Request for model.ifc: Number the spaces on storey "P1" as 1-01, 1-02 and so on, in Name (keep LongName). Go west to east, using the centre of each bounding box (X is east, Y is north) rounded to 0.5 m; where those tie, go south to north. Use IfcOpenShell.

First a look at what the model holds.

```python
import ifcopenshell
import ifcopenshell.util.element
import ifcopenshell.util.placement

model = ifcopenshell.open("model.ifc")
print(model.schema)
storey = next(s for s in model.by_type("IfcBuildingStorey") if s.Name == "P1")
spaces = [e for e in ifcopenshell.util.element.get_decomposition(storey) if e.is_a("IfcSpace")]
for e in sorted(spaces, key=lambda e: e.id()):
    origin = ifcopenshell.util.placement.get_local_placement(e.ObjectPlacement)[:3, 3]
    print(e.id(), e.Name, e.LongName, origin.round(2) + 0.0, sep=" | ")
```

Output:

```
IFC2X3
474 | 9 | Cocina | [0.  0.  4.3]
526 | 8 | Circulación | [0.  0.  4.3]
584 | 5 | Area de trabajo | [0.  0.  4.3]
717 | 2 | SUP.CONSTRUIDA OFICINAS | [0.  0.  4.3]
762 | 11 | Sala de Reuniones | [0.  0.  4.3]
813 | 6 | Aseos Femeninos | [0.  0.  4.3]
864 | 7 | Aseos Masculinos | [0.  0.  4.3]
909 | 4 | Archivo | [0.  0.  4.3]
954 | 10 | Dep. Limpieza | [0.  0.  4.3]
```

```python
import ifcopenshell
import ifcopenshell.geom
import ifcopenshell.util.element
import ifcopenshell.util.shape

model = ifcopenshell.open("model.ifc")
settings = ifcopenshell.geom.settings()
settings.set("use-world-coords", True)


def centre(element):
    shape = ifcopenshell.geom.create_shape(settings, element)
    return ifcopenshell.util.shape.get_bbox_centroid(shape.geometry)


storey = next(s for s in model.by_type("IfcBuildingStorey") if s.Name == "P1")
spaces = [e for e in ifcopenshell.util.element.get_decomposition(storey) if e.is_a("IfcSpace")]

# Insertion points can sit at a corner or the storey origin, so sort by the geometry (in metres).
centres = {e: centre(e) for e in spaces}
spaces.sort(key=lambda e: (round(centres[e][0] / 0.5), centres[e][1]))

for i, e in enumerate(spaces, start=1):
    number = f"1-{i:02d}"
    e.Name = number
    print(e.id(), number)

model.write("model_updated.ifc")
```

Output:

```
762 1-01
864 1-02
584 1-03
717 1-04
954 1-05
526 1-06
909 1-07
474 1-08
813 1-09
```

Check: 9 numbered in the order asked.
